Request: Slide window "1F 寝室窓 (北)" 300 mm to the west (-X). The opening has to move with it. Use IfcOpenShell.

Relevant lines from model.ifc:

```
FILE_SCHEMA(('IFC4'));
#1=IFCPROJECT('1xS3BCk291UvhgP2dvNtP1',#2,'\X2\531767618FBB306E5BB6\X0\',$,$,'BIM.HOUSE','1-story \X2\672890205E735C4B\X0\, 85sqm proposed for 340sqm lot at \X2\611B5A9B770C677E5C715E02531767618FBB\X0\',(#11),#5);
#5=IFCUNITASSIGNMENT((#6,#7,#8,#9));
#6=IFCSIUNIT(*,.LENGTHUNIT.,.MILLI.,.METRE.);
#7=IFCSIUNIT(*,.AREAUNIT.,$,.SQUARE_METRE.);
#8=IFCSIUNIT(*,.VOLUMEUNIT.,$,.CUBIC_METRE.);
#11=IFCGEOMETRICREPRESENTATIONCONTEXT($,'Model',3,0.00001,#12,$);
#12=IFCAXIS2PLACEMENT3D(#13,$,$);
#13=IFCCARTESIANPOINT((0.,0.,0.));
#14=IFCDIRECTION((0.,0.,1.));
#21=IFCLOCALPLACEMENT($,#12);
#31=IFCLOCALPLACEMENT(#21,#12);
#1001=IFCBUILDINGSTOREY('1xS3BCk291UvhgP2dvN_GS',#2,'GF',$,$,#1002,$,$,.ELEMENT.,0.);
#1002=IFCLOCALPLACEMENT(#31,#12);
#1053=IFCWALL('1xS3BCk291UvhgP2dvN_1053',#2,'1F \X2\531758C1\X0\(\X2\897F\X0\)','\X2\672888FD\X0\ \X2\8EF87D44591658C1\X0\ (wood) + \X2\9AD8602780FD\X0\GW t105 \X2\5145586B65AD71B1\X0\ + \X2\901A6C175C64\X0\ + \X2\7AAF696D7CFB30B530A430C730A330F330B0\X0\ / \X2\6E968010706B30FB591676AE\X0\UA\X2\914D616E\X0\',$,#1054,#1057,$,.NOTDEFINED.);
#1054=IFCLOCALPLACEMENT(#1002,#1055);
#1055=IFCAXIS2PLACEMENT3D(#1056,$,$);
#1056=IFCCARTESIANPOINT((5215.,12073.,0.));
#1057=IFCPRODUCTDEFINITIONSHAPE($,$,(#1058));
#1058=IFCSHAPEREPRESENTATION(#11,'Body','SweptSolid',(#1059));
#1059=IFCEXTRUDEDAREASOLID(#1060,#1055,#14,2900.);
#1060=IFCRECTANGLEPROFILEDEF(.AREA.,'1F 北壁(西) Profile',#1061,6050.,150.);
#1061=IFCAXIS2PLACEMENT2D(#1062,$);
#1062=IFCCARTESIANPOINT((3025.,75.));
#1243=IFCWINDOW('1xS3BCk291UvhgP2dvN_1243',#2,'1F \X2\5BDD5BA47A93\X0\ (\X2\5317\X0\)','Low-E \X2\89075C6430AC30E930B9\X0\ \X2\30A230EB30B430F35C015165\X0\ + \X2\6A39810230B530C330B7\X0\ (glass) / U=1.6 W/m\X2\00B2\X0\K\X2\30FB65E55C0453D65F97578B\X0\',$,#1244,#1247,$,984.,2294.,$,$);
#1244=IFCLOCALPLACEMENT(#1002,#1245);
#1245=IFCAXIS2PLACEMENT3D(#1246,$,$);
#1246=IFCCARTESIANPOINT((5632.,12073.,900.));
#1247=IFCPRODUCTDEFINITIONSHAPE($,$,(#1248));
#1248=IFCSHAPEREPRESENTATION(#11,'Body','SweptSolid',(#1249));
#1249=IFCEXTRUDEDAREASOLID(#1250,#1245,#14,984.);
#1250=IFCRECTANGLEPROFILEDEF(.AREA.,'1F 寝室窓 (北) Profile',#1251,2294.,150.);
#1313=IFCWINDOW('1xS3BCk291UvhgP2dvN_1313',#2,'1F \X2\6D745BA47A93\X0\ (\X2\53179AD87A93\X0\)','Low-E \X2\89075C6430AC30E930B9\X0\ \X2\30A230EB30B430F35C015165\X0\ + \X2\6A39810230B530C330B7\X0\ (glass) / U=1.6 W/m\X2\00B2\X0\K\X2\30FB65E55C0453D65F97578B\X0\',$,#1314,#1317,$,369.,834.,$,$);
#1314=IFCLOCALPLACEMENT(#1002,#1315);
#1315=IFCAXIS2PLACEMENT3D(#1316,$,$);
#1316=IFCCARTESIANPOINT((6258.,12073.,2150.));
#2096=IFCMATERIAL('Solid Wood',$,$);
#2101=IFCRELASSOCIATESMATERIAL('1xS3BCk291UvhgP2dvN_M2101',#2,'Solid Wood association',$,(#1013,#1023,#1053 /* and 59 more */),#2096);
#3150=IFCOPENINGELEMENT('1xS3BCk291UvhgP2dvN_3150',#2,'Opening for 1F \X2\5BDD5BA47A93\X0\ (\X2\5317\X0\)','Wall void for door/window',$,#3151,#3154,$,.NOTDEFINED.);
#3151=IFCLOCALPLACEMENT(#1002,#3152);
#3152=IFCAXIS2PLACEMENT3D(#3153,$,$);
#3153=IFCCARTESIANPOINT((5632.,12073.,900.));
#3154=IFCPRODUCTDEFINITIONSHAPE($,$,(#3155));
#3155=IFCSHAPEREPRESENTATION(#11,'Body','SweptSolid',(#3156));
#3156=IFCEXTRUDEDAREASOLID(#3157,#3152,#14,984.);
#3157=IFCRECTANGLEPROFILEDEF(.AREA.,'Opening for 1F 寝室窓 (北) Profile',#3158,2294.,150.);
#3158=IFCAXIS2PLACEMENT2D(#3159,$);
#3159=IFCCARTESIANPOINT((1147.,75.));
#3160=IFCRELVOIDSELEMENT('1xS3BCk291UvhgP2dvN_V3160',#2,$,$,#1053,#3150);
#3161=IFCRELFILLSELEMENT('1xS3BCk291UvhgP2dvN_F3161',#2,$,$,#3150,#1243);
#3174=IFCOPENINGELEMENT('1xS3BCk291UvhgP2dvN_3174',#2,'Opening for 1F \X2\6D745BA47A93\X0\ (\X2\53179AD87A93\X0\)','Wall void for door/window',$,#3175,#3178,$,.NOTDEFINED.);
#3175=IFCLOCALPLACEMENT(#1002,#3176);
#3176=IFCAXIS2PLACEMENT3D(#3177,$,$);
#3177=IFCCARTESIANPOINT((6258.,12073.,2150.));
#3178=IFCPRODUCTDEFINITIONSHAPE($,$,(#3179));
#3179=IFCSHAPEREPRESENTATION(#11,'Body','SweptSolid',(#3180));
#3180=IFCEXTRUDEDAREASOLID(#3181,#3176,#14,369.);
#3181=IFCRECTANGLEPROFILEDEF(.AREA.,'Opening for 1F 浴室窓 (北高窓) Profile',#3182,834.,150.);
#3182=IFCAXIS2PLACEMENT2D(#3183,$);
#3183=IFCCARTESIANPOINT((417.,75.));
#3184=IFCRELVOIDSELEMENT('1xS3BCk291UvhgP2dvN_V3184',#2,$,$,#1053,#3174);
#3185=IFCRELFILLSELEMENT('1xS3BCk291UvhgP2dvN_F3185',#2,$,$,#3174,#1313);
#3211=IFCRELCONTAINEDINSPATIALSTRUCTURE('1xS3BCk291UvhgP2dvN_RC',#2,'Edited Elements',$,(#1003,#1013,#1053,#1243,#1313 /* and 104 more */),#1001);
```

```python
import ifcopenshell
import ifcopenshell.api.geometry
import ifcopenshell.util.placement
import ifcopenshell.util.unit

model = ifcopenshell.open("model.ifc")
unit_scale = ifcopenshell.util.unit.calculate_unit_scale(model)

window = model.by_guid("1xS3BCk291UvhgP2dvN_1243")
opening = window.FillsVoids[0].RelatingOpeningElement
wall = opening.VoidsElements[0].RelatingBuildingElement

wall_matrix = ifcopenshell.util.placement.get_local_placement(wall.ObjectPlacement)
shift = wall_matrix[:3, 0] * -0.3 / unit_scale
before = ifcopenshell.util.placement.get_local_placement(window.ObjectPlacement)[:3, 3].copy()

# The window is not placed relative to its opening, so move both.
for product in (opening, window):
    matrix = ifcopenshell.util.placement.get_local_placement(product.ObjectPlacement)
    matrix[:3, 3] += shift
    ifcopenshell.api.geometry.edit_object_placement(model, product=product, matrix=matrix, is_si=False)

after = ifcopenshell.util.placement.get_local_placement(window.ObjectPlacement)[:3, 3]
print("window moved by", (after - before).round(3) + 0.0)

model.write("model_v2.ifc")
```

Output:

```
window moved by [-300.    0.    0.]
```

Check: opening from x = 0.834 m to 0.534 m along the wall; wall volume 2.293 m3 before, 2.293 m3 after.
